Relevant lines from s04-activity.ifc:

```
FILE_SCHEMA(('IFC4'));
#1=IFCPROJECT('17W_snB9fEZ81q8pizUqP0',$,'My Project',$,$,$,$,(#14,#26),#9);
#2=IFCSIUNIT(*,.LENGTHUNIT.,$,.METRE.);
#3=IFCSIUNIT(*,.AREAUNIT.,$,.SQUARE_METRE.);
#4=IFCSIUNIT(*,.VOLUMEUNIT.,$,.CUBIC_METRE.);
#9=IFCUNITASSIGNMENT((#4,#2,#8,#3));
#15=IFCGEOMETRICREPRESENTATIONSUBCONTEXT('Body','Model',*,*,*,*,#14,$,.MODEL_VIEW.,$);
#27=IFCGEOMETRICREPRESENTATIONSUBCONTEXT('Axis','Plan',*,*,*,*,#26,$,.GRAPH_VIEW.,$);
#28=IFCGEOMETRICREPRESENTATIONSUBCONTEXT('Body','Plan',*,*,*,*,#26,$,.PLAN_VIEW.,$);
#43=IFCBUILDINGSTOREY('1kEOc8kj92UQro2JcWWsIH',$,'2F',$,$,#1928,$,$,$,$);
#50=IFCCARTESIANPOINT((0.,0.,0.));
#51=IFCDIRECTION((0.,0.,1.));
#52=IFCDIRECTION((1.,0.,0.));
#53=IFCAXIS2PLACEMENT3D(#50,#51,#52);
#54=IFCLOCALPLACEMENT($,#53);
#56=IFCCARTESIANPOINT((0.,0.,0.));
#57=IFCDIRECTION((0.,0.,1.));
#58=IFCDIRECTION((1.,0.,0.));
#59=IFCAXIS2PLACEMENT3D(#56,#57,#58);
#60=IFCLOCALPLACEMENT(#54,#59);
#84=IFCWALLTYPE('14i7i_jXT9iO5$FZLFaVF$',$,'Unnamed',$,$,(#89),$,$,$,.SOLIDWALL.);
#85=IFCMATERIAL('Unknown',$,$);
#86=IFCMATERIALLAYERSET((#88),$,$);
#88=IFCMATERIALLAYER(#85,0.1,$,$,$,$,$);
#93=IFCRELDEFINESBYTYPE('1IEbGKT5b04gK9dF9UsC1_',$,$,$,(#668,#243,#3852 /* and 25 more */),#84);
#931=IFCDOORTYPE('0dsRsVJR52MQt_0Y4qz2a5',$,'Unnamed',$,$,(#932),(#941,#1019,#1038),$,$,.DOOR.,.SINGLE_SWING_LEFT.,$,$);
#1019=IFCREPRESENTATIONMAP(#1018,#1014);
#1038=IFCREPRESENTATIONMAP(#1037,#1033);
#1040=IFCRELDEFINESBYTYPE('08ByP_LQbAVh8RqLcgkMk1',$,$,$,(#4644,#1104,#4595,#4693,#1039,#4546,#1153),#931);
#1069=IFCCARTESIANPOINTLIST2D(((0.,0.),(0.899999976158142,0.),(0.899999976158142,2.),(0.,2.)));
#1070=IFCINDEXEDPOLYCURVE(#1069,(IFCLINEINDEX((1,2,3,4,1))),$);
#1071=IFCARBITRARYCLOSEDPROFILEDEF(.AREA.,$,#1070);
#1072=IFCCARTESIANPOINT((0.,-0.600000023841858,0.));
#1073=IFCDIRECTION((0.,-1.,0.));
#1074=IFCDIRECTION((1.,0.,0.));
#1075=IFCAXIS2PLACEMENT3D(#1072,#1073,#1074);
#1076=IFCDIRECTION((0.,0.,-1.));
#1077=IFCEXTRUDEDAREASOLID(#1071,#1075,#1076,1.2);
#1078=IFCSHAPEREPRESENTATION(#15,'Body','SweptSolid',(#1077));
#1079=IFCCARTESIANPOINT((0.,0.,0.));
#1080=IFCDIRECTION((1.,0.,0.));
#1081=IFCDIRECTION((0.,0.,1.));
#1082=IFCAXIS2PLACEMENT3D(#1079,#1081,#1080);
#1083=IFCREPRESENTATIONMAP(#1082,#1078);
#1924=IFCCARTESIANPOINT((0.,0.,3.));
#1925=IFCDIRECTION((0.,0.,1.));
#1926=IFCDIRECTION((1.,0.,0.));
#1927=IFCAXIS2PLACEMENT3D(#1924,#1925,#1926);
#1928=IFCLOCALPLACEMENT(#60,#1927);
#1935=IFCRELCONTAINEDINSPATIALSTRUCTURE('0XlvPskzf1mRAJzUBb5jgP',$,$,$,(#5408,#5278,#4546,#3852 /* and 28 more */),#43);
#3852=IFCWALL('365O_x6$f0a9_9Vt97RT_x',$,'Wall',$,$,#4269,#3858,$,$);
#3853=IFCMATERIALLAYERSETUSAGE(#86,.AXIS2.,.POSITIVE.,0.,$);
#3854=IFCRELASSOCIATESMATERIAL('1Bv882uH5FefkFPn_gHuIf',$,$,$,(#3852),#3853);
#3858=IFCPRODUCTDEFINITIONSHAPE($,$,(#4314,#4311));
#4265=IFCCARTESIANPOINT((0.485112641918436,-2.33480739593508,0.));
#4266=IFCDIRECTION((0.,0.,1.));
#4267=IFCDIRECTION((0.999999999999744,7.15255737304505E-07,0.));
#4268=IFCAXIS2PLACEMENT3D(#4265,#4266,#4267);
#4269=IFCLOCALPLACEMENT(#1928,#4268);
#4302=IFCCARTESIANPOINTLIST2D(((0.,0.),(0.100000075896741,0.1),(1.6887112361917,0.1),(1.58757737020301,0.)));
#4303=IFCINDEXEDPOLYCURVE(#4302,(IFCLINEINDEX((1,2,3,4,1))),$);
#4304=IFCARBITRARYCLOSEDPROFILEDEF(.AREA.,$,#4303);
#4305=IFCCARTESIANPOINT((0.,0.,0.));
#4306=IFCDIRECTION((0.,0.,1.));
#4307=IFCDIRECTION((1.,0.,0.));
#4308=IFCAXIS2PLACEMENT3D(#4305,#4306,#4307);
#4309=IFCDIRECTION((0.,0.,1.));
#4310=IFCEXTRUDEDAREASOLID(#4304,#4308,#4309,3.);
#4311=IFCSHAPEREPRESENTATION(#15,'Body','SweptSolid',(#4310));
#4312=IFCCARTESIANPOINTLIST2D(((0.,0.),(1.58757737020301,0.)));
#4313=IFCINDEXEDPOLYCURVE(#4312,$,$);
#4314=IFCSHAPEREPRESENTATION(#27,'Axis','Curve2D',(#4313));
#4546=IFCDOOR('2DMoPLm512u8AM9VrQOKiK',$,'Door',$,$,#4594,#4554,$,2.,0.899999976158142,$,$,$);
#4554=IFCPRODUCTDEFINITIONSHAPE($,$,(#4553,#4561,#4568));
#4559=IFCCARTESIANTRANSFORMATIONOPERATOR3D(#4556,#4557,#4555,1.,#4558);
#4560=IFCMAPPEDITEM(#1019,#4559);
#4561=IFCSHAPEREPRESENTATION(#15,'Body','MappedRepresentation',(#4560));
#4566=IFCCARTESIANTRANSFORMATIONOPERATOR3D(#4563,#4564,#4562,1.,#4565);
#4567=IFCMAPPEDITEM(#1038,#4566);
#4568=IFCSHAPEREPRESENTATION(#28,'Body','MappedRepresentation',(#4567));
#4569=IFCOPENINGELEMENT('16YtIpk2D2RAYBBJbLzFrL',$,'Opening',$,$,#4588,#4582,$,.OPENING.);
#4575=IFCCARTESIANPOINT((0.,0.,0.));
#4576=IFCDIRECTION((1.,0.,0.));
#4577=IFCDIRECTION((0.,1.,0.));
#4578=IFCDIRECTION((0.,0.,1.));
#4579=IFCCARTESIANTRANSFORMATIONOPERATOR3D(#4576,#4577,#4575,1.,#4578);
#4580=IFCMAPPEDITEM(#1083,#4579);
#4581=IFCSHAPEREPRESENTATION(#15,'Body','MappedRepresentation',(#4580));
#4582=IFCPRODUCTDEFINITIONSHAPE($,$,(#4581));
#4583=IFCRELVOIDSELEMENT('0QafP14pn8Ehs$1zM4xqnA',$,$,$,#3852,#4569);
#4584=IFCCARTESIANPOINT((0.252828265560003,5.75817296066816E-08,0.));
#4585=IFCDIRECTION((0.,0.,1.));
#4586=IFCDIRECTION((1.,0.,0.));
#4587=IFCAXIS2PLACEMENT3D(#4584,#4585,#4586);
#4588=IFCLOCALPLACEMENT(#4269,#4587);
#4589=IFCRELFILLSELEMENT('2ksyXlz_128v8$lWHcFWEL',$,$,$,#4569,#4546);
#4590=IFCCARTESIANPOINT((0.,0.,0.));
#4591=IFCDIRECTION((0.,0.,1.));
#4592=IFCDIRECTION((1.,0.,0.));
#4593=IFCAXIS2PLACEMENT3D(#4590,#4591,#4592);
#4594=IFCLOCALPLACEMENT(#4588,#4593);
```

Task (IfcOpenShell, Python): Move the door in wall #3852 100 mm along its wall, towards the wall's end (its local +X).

```python
import ifcopenshell
import ifcopenshell.api.geometry
import ifcopenshell.util.placement

model = ifcopenshell.open("s04-activity.ifc")

door = model.by_guid("2DMoPLm512u8AM9VrQOKiK")
opening = door.FillsVoids[0].RelatingOpeningElement
wall = opening.VoidsElements[0].RelatingBuildingElement

wall_matrix = ifcopenshell.util.placement.get_local_placement(wall.ObjectPlacement)
shift = wall_matrix[:3, 0] * 0.1
before = ifcopenshell.util.placement.get_local_placement(door.ObjectPlacement)[:3, 3].copy()

# The door is placed relative to its opening, so it follows when the opening moves.
matrix = ifcopenshell.util.placement.get_local_placement(opening.ObjectPlacement)
matrix[:3, 3] += shift
ifcopenshell.api.geometry.edit_object_placement(
    model, product=opening, matrix=matrix, is_si=False, should_transform_children=True
)

after = ifcopenshell.util.placement.get_local_placement(door.ObjectPlacement)[:3, 3]
print("door moved by", (after - before).round(3) + 0.0)

model.write("s04-activity_rev.ifc")
```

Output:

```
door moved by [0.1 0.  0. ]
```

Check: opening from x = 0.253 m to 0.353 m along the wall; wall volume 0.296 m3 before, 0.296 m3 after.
